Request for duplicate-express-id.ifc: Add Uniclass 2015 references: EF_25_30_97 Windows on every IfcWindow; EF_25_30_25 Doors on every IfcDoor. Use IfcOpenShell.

First a look at what the model holds.

```python
import ifcopenshell

model = ifcopenshell.open("duplicate-express-id.ifc")
print(model.schema)
print("classifications:", [c.Name for c in model.by_type("IfcClassification")])
for ifc_class in ("IfcDoor", "IfcRoof", "IfcStair", "IfcWall", "IfcWindow"):
    print(ifc_class, len(model.by_type(ifc_class)))
```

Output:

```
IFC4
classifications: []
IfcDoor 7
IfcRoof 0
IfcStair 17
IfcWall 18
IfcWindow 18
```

```python
import ifcopenshell
import ifcopenshell.api.classification

model = ifcopenshell.open("duplicate-express-id.ifc")

system = ifcopenshell.api.classification.add_classification(model, classification="Uniclass 2015")

codes = {
    "IfcWindow": ("EF_25_30_97", "Windows"),
    "IfcDoor": ("EF_25_30_25", "Doors"),
}
for ifc_class, (code, name) in codes.items():
    products = model.by_type(ifc_class)
    ifcopenshell.api.classification.add_reference(
        model, products=products, classification=system, identification=code, name=name
    )
    print(code, len(products))

model.write("duplicate-express-id_updated.ifc")
```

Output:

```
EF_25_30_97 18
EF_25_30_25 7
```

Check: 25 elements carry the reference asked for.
